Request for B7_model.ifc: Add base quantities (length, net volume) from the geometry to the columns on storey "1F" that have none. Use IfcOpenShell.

First a look at what the model holds.

```python
import ifcopenshell
import ifcopenshell.util.element
import ifcopenshell.util.unit

model = ifcopenshell.open("B7_model.ifc")
print(model.schema)
for unit_type in ("LENGTHUNIT", "AREAUNIT", "VOLUMEUNIT"):
    print(unit_type, ifcopenshell.util.unit.calculate_unit_scale(model, unit_type))
storey = next(s for s in model.by_type("IfcBuildingStorey") if s.Name == "1F")
columns = [e for e in ifcopenshell.util.element.get_decomposition(storey) if e.is_a("IfcColumn")]
for e in sorted(columns, key=lambda e: e.id()):
    print(e.id(), e.is_a(), e.Name, list(ifcopenshell.util.element.get_psets(e, qtos_only=True)), sep=" | ")
```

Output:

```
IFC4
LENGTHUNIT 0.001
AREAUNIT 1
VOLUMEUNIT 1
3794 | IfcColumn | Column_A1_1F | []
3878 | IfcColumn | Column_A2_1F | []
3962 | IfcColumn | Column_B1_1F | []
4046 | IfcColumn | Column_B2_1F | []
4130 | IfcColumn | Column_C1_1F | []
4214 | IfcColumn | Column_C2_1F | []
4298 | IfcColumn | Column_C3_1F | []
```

```python
import ifcopenshell
import ifcopenshell.api.pset
import ifcopenshell.geom
import ifcopenshell.util.element
import ifcopenshell.util.shape
import ifcopenshell.util.unit

model = ifcopenshell.open("B7_model.ifc")
unit_scale = ifcopenshell.util.unit.calculate_unit_scale(model)
volume_scale = ifcopenshell.util.unit.calculate_unit_scale(model, "VOLUMEUNIT")
settings = ifcopenshell.geom.settings()

storey = next(s for s in model.by_type("IfcBuildingStorey") if s.Name == "1F")
columns = [e for e in ifcopenshell.util.element.get_decomposition(storey) if e.is_a("IfcColumn")]

for e in sorted(columns, key=lambda e: e.id()):
    if ifcopenshell.util.element.get_psets(e, qtos_only=True, should_inherit=False):
        continue
    # Geometry comes back in metres, in the element's own axes.
    shape = ifcopenshell.geom.create_shape(settings, e)
    values = {
        "Length": ifcopenshell.util.shape.get_z(shape.geometry) / unit_scale,
        "NetVolume": ifcopenshell.util.shape.get_volume(shape.geometry) / volume_scale,
    }
    qto = ifcopenshell.api.pset.add_qto(model, product=e, name="Qto_ColumnBaseQuantities")
    ifcopenshell.api.pset.edit_qto(model, qto=qto, properties=values)
    print(e.id(), {k: round(v, 3) for k, v in values.items()})

model.write("B7_model_rev.ifc")
```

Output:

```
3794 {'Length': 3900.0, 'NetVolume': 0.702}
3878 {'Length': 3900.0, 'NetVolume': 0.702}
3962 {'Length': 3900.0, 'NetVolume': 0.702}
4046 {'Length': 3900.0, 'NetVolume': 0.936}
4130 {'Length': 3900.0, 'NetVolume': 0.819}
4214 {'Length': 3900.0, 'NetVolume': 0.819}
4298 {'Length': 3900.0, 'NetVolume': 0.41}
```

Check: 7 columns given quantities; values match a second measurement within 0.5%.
